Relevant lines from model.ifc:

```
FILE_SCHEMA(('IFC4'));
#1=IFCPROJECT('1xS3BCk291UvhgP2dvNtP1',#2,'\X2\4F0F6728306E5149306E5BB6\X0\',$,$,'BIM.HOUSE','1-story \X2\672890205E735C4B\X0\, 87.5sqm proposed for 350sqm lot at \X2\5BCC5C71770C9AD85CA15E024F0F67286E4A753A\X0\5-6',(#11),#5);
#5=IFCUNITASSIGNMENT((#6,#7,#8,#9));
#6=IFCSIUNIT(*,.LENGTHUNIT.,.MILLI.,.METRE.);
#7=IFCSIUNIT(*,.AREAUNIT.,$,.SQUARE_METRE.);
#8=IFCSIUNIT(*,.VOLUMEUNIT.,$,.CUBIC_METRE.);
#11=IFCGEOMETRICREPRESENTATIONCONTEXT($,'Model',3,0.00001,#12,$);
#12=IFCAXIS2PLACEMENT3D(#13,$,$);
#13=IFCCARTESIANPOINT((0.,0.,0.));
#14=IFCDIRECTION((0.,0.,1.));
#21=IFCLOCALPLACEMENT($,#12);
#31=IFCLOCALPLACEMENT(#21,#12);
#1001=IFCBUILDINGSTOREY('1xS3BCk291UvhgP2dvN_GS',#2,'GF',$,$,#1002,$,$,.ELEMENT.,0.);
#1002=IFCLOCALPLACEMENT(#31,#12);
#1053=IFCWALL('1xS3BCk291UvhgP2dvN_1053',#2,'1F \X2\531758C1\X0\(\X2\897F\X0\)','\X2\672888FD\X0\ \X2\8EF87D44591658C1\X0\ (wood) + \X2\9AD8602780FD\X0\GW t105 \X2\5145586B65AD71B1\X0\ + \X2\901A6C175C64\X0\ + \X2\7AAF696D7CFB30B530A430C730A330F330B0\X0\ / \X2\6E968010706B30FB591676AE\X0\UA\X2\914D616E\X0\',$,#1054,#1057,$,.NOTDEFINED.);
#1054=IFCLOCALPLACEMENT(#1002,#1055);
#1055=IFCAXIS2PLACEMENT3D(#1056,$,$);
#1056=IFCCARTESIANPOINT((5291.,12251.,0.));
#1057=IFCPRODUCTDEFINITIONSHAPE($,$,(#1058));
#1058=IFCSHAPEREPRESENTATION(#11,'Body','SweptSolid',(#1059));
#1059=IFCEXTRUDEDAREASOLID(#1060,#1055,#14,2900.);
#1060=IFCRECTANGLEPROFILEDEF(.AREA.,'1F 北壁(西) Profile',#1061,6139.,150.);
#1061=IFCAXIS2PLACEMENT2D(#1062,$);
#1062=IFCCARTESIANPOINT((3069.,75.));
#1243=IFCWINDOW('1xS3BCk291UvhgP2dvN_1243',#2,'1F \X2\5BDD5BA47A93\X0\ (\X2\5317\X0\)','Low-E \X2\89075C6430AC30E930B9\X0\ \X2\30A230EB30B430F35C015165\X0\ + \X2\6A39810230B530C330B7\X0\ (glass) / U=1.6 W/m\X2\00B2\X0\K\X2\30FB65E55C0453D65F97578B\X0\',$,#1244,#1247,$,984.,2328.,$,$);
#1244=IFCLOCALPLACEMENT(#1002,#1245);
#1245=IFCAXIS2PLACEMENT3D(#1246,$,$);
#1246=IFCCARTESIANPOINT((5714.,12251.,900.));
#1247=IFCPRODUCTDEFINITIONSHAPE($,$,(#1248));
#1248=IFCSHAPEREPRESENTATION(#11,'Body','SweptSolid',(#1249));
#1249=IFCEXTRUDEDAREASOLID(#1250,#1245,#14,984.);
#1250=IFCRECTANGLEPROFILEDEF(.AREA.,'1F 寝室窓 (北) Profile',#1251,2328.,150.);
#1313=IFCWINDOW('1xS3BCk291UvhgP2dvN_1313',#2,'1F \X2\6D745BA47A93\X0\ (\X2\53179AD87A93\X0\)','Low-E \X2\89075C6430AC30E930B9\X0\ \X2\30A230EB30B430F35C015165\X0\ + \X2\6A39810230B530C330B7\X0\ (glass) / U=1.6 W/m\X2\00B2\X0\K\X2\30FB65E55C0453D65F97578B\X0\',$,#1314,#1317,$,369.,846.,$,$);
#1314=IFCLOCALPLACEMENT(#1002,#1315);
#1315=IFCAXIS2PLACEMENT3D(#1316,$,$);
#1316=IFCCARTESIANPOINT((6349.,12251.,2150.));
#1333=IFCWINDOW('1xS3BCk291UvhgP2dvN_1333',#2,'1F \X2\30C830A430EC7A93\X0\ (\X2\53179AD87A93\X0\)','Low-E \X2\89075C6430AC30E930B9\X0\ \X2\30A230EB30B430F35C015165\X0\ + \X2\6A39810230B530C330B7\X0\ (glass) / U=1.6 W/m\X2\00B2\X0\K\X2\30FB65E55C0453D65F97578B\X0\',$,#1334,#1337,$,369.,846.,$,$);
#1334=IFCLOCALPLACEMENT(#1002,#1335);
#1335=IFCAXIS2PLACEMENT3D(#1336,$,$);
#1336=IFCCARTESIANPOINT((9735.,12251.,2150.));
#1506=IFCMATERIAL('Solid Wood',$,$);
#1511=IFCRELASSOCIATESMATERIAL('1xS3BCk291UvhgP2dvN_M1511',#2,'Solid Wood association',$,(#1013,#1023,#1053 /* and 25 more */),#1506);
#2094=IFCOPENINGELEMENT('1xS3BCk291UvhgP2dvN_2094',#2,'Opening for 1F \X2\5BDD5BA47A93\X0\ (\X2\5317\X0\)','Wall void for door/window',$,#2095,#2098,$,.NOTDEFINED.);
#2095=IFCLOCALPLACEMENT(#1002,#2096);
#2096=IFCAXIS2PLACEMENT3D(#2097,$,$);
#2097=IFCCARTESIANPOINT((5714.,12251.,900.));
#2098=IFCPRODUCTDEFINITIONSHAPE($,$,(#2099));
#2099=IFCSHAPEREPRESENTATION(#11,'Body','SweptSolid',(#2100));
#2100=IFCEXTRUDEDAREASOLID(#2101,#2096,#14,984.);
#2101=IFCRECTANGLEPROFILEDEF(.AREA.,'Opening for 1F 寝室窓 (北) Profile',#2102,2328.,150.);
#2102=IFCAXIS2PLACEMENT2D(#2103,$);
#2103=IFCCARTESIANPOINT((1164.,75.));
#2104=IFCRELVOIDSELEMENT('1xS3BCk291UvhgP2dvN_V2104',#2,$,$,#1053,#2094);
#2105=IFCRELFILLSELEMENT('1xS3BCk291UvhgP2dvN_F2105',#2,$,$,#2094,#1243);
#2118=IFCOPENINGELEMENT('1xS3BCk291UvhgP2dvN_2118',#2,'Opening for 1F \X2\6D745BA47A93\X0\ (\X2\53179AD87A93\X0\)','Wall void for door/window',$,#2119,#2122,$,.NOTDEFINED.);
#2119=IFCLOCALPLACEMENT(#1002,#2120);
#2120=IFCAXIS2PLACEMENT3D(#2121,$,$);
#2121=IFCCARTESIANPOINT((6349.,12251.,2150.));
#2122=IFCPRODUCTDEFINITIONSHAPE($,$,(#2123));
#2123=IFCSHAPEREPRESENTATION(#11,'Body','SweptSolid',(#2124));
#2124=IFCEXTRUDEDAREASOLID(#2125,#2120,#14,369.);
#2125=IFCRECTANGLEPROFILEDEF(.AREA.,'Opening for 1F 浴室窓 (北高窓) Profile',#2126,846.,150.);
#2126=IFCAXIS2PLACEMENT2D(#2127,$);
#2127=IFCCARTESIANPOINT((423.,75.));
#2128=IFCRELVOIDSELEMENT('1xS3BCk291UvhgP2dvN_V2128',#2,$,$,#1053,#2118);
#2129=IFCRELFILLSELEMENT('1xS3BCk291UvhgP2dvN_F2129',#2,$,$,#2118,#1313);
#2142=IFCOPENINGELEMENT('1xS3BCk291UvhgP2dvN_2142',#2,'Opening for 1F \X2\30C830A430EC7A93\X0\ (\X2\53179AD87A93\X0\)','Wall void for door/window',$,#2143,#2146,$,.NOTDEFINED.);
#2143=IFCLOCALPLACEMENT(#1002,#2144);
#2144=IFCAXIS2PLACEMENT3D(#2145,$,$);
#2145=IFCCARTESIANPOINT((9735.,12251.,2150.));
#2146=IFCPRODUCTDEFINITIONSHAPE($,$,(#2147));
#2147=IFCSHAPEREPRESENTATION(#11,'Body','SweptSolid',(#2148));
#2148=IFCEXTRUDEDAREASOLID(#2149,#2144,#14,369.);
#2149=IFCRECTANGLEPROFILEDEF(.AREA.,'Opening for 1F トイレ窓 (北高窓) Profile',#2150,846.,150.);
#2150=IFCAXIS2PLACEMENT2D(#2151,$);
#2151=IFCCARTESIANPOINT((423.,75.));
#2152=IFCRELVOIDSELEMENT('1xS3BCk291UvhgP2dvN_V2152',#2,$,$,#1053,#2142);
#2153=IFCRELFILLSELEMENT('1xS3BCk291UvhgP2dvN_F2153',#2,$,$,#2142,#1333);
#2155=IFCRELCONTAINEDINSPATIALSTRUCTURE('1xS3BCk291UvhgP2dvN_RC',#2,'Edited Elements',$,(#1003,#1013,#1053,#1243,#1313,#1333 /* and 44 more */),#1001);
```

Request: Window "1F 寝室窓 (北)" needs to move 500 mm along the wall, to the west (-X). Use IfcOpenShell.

```python
import ifcopenshell
import ifcopenshell.api.geometry
import ifcopenshell.util.placement

model = ifcopenshell.open("model.ifc")

window = model.by_id(1243)
opening = window.FillsVoids[0].RelatingOpeningElement
wall = opening.VoidsElements[0].RelatingBuildingElement

wall_matrix = ifcopenshell.util.placement.get_local_placement(wall.ObjectPlacement)
shift = wall_matrix[:3, 0] * -500.0
before = ifcopenshell.util.placement.get_local_placement(window.ObjectPlacement)[:3, 3].copy()

# The window is not placed relative to its opening, so move both.
for product in (opening, window):
    matrix = ifcopenshell.util.placement.get_local_placement(product.ObjectPlacement)
    matrix[:3, 3] += shift
    ifcopenshell.api.geometry.edit_object_placement(model, product=product, matrix=matrix, is_si=False)

after = ifcopenshell.util.placement.get_local_placement(window.ObjectPlacement)[:3, 3]
print("window moved by", (after - before).round(3) + 0.0)

model.write("model_rev.ifc")
```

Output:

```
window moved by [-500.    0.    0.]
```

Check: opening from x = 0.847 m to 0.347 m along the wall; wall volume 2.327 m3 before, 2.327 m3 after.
